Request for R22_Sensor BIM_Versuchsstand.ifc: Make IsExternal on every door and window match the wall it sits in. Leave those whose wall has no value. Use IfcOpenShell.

First a look at what the model holds.

```python
import ifcopenshell
import ifcopenshell.util.element

model = ifcopenshell.open("R22_Sensor BIM_Versuchsstand.ifc")
print(model.schema)
seen = {}
for e in model.by_type("IfcDoor") + model.by_type("IfcWindow"):
    if not e.FillsVoids:
        continue
    host = e.FillsVoids[0].RelatingOpeningElement.VoidsElements[0].RelatingBuildingElement
    own = ifcopenshell.util.element.get_pset(e, f"Pset_{e.is_a()[3:].removesuffix('StandardCase')}Common", "IsExternal")
    wall = ifcopenshell.util.element.get_pset(host, "Pset_WallCommon", "IsExternal")
    seen[e.is_a(), own, wall] = seen.get((e.is_a(), own, wall), 0) + 1
for (cls, own, wall), count in sorted(seen.items(), key=str):
    print(count, cls, "IsExternal:", own, "| host wall:", wall)
```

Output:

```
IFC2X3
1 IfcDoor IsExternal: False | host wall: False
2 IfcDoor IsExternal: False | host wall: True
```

```python
import ifcopenshell
import ifcopenshell.api.pset
import ifcopenshell.util.element

model = ifcopenshell.open("R22_Sensor BIM_Versuchsstand.ifc")

count = 0
for ifc_class, pset_name in (("IfcDoor", "Pset_DoorCommon"), ("IfcWindow", "Pset_WindowCommon")):
    for e in model.by_type(ifc_class):
        if not e.FillsVoids:
            continue
        host = e.FillsVoids[0].RelatingOpeningElement.VoidsElements[0].RelatingBuildingElement
        external = ifcopenshell.util.element.get_pset(host, "Pset_WallCommon", "IsExternal")
        if external is None or ifcopenshell.util.element.get_pset(e, pset_name, "IsExternal") == external:
            continue
        pset = ifcopenshell.api.pset.add_pset(model, product=e, name=pset_name)
        ifcopenshell.api.pset.edit_pset(model, pset=pset, properties={"IsExternal": external})
        count += 1

print(count, "updated")

model.write("R22_Sensor BIM_Versuchsstand_edited.ifc")
```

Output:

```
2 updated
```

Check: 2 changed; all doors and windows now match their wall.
